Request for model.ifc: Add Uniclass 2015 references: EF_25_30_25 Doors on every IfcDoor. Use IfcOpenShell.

First a look at what the model holds.

```python
import ifcopenshell

model = ifcopenshell.open("model.ifc")
print(model.schema)
print("classifications:", [c.Name for c in model.by_type("IfcClassification")])
for ifc_class in ("IfcDoor", "IfcRoof", "IfcStair", "IfcWall", "IfcWindow"):
    print(ifc_class, len(model.by_type(ifc_class)))
```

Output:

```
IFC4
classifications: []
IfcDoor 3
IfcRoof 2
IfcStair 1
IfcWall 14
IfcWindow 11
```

```python
import ifcopenshell
import ifcopenshell.api.classification

model = ifcopenshell.open("model.ifc")

system = ifcopenshell.api.classification.add_classification(model, classification="Uniclass 2015")

codes = {
    "IfcDoor": ("EF_25_30_25", "Doors"),
}
for ifc_class, (code, name) in codes.items():
    products = model.by_type(ifc_class)
    ifcopenshell.api.classification.add_reference(
        model, products=products, classification=system, identification=code, name=name
    )
    print(code, len(products))

model.write("model_rev.ifc")
```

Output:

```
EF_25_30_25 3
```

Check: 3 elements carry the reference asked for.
